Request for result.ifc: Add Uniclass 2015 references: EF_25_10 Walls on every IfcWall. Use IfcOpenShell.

First a look at what the model holds.

```python
import ifcopenshell

model = ifcopenshell.open("result.ifc")
print(model.schema)
print("classifications:", [c.Name for c in model.by_type("IfcClassification")])
for ifc_class in ("IfcDoor", "IfcRoof", "IfcStair", "IfcWall", "IfcWindow"):
    print(ifc_class, len(model.by_type(ifc_class)))
```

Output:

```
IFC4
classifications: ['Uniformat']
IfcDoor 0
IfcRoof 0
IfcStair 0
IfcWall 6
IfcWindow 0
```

```python
import ifcopenshell
import ifcopenshell.api.classification

model = ifcopenshell.open("result.ifc")

system = ifcopenshell.api.classification.add_classification(model, classification="Uniclass 2015")

codes = {
    "IfcWall": ("EF_25_10", "Walls"),
}
for ifc_class, (code, name) in codes.items():
    products = model.by_type(ifc_class)
    ifcopenshell.api.classification.add_reference(
        model, products=products, classification=system, identification=code, name=name
    )
    print(code, len(products))

model.write("result_rev.ifc")
```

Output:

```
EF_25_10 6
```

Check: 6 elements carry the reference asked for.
